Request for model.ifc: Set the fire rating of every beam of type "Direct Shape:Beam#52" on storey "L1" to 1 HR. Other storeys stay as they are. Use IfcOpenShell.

First a look at what the model holds.

```python
import ifcopenshell
import ifcopenshell.util.element

model = ifcopenshell.open("model.ifc")
print(model.schema)
storey = next(s for s in model.by_type("IfcBuildingStorey") if s.Name == "L1")
beams = [e for e in ifcopenshell.util.element.get_decomposition(storey) if e.is_a("IfcBeam")]
seen = {}
for e in beams:
    element_type = ifcopenshell.util.element.get_type(e)
    key = (element_type.Name if element_type != e and element_type else None, ifcopenshell.util.element.get_pset(e, "Pset_BeamCommon", "FireRating"))
    seen[key] = seen.get(key, 0) + 1
for (name, value), count in sorted(seen.items(), key=str):
    print(count, "x", name, "|", value)
```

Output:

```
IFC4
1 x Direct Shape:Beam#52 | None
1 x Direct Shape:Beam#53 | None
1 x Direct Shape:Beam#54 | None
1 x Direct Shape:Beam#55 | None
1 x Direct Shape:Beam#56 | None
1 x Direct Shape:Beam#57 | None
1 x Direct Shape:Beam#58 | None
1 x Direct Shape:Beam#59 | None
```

```python
import ifcopenshell
import ifcopenshell.api.pset
import ifcopenshell.util.element

model = ifcopenshell.open("model.ifc")

storey = next(s for s in model.by_type("IfcBuildingStorey") if s.Name == "L1")
beams = [e for e in ifcopenshell.util.element.get_decomposition(storey) if e.is_a("IfcBeam")]

count = 0
for e in beams:
    element_type = ifcopenshell.util.element.get_type(e)
    if element_type in (None, e) or element_type.Name != "Direct Shape:Beam#52":
        continue
    # add_pset returns the element's existing set when there is one.
    pset = ifcopenshell.api.pset.add_pset(model, product=e, name="Pset_BeamCommon")
    ifcopenshell.api.pset.edit_pset(model, pset=pset, properties={"FireRating": "1 HR"})
    count += 1

print(count, "beams updated")

model.write("model-out.ifc")
```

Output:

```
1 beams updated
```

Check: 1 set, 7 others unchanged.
